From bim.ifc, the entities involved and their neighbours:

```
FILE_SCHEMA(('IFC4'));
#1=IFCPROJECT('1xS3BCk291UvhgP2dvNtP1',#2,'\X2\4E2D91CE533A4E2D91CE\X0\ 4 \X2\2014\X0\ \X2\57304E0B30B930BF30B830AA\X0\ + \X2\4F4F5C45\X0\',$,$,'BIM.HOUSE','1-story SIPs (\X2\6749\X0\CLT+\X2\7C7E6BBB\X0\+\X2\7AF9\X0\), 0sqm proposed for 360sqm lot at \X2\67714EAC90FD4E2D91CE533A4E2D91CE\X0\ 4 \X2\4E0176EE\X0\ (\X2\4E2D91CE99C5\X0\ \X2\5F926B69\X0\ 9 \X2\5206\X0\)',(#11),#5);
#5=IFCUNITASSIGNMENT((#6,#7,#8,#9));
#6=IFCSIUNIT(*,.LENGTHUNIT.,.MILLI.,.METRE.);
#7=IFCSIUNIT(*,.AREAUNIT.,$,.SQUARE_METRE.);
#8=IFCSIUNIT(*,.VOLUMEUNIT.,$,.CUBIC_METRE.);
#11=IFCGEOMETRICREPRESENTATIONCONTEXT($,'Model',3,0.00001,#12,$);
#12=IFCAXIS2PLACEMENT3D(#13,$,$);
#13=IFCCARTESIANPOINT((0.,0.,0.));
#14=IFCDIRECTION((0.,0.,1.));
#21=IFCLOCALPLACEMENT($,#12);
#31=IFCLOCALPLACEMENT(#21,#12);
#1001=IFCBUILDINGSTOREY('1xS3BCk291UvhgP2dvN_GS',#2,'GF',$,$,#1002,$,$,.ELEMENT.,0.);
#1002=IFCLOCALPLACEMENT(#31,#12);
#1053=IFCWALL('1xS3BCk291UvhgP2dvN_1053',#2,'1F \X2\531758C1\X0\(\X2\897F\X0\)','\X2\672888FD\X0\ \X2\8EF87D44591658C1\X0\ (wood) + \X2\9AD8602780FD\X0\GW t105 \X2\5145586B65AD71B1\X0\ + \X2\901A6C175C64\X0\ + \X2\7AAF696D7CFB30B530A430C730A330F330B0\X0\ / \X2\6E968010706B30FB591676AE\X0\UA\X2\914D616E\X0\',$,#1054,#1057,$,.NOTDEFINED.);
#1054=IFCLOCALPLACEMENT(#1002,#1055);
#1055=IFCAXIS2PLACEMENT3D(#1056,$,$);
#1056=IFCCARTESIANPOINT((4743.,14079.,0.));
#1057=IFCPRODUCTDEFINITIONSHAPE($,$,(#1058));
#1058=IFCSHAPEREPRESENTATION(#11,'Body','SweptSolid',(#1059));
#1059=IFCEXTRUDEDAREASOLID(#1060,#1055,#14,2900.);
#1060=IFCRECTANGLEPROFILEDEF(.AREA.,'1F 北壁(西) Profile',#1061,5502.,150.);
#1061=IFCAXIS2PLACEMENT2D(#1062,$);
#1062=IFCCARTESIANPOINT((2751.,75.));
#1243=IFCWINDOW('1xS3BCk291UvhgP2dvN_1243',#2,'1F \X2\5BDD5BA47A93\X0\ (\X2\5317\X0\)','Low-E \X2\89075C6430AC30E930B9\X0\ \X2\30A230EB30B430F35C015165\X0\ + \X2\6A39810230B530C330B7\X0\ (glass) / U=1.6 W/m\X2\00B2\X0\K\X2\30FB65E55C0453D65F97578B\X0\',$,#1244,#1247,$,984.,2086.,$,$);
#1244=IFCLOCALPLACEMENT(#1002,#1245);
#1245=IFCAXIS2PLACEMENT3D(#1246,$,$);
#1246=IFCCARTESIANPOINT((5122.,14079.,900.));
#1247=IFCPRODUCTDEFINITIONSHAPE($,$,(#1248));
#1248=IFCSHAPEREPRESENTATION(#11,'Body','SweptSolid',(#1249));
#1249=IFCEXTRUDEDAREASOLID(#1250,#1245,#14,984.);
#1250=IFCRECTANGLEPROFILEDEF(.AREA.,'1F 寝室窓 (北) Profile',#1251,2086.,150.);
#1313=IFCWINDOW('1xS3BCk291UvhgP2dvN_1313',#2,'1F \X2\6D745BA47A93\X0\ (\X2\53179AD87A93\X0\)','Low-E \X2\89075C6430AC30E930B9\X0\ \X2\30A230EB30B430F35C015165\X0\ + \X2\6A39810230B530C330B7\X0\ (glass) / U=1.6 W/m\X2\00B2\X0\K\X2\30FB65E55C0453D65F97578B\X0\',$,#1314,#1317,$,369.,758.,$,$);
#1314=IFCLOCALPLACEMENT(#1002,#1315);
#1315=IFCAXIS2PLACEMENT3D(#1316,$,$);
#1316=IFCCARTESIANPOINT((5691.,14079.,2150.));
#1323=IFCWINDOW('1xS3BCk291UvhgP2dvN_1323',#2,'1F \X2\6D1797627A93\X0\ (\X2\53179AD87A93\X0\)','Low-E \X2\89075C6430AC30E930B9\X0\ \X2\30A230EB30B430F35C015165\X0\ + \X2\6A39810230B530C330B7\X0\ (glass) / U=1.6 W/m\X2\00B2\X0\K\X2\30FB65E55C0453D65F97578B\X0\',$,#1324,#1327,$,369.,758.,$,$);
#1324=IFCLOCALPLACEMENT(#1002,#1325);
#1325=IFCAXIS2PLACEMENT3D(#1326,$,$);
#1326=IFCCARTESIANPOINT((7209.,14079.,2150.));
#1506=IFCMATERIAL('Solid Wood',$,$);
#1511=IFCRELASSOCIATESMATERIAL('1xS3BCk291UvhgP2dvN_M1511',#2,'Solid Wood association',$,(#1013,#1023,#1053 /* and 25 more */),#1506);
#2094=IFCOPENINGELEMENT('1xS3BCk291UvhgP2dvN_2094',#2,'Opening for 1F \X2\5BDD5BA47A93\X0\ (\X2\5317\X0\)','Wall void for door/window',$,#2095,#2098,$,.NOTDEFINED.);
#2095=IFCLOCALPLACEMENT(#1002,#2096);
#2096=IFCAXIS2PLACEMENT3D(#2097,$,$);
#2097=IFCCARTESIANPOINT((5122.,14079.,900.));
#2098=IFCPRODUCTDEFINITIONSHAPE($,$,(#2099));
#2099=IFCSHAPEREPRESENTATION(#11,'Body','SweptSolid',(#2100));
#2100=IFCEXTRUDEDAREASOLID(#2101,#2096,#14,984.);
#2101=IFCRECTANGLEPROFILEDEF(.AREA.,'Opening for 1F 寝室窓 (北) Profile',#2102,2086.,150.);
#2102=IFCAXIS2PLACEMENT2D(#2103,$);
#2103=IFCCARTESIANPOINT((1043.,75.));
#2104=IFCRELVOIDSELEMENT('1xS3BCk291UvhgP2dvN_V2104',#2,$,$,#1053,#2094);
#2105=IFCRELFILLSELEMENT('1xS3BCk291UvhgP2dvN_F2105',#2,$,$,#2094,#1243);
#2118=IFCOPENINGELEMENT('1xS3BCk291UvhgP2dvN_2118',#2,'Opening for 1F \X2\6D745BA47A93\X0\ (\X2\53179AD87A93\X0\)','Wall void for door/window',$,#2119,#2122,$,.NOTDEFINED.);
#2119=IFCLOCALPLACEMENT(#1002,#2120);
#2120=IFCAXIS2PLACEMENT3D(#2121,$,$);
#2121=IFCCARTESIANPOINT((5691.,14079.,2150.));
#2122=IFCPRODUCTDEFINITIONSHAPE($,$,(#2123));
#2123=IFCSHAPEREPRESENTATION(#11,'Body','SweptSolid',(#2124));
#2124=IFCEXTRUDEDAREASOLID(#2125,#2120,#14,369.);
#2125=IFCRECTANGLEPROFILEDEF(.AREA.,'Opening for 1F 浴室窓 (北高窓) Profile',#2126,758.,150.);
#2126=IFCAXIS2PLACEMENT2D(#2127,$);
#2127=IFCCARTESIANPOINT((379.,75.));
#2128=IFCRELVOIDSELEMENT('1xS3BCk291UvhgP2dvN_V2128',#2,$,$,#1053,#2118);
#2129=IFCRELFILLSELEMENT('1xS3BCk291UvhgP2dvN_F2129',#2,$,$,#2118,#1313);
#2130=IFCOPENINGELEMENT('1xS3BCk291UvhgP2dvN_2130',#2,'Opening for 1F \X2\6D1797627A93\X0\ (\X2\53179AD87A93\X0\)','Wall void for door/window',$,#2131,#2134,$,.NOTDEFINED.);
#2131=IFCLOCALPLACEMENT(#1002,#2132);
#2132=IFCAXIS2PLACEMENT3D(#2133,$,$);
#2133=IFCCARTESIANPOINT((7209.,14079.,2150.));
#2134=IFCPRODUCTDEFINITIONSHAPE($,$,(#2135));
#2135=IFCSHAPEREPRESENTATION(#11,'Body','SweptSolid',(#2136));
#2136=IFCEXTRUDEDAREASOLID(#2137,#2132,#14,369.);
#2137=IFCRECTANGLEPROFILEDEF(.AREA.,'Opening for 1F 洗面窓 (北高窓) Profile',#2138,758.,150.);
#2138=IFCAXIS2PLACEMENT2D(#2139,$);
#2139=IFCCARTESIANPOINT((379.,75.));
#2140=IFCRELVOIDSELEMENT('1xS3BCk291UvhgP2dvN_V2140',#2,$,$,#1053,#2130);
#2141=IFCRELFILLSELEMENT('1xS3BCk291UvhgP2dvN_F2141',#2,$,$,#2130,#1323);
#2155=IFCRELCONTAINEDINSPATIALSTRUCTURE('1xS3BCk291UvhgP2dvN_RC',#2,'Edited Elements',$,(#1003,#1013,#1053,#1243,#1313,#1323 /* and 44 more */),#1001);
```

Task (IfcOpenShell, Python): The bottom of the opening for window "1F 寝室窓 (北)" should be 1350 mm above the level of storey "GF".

```python
import numpy as np
import ifcopenshell
import ifcopenshell.api.geometry
import ifcopenshell.geom
import ifcopenshell.util.element
import ifcopenshell.util.placement
import ifcopenshell.util.shape
import ifcopenshell.util.unit

model = ifcopenshell.open("bim.ifc")
unit_scale = ifcopenshell.util.unit.calculate_unit_scale(model)

window = model.by_guid("1xS3BCk291UvhgP2dvN_1243")
opening = window.FillsVoids[0].RelatingOpeningElement
storey = ifcopenshell.util.element.get_container(window, ifc_class="IfcBuildingStorey")
level = ifcopenshell.util.placement.get_local_placement(storey.ObjectPlacement)[2, 3]

# The opening's origin need not be at the sill, so measure its lowest point.
shape = ifcopenshell.geom.create_shape(ifcopenshell.geom.settings(), opening)
bottom = ifcopenshell.util.shape.get_shape_bottom_elevation(shape, shape.geometry) / unit_scale
dz = level + 1.35 / unit_scale - bottom

shift = np.array([0.0, 0.0, dz])
# The window is not placed relative to its opening, so move both.
for product in (opening, window):
    matrix = ifcopenshell.util.placement.get_local_placement(product.ObjectPlacement)
    matrix[:3, 3] += shift
    ifcopenshell.api.geometry.edit_object_placement(model, product=product, matrix=matrix, is_si=False)

print(f"moved by {dz * unit_scale:+.3f} m")

model.write("bim_updated.ifc")
```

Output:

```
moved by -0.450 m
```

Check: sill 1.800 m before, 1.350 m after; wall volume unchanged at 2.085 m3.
